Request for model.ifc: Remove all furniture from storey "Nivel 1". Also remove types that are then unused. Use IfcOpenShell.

First a look at what the model holds.

```python
import ifcopenshell
import ifcopenshell.util.element

model = ifcopenshell.open("model.ifc")
print(model.schema)
storey = next(s for s in model.by_type("IfcBuildingStorey") if s.Name == "Nivel 1")
furniture = [e for e in ifcopenshell.util.element.get_decomposition(storey) if e.is_a("IfcFurnishingElement")]
seen = {}
for e in furniture:
    element_type = ifcopenshell.util.element.get_type(e)
    name = element_type.Name if element_type not in (None, e) else None
    seen[name] = seen.get(name, 0) + 1
for name, count in sorted(seen.items(), key=str):
    print(count, "x", name)
```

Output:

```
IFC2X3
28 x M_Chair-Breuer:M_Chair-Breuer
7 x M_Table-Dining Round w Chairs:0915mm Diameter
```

```python
import ifcopenshell
import ifcopenshell.api.root
import ifcopenshell.util.element

model = ifcopenshell.open("model.ifc")

storey = next(s for s in model.by_type("IfcBuildingStorey") if s.Name == "Nivel 1")
furniture = [e for e in ifcopenshell.util.element.get_decomposition(storey) if e.is_a("IfcFurnishingElement")]
types = {ifcopenshell.util.element.get_type(e) for e in furniture} - {None, *furniture}

for e in furniture:
    ifcopenshell.api.root.remove_product(model, product=e)
print(len(furniture), "removed")

unused = [t for t in types if not ifcopenshell.util.element.get_types(t)]
for t in unused:
    ifcopenshell.api.root.remove_product(model, product=t)
print(len(unused), "unused types removed")

model.write("model-out.ifc")
```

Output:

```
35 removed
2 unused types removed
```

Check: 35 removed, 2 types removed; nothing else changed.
